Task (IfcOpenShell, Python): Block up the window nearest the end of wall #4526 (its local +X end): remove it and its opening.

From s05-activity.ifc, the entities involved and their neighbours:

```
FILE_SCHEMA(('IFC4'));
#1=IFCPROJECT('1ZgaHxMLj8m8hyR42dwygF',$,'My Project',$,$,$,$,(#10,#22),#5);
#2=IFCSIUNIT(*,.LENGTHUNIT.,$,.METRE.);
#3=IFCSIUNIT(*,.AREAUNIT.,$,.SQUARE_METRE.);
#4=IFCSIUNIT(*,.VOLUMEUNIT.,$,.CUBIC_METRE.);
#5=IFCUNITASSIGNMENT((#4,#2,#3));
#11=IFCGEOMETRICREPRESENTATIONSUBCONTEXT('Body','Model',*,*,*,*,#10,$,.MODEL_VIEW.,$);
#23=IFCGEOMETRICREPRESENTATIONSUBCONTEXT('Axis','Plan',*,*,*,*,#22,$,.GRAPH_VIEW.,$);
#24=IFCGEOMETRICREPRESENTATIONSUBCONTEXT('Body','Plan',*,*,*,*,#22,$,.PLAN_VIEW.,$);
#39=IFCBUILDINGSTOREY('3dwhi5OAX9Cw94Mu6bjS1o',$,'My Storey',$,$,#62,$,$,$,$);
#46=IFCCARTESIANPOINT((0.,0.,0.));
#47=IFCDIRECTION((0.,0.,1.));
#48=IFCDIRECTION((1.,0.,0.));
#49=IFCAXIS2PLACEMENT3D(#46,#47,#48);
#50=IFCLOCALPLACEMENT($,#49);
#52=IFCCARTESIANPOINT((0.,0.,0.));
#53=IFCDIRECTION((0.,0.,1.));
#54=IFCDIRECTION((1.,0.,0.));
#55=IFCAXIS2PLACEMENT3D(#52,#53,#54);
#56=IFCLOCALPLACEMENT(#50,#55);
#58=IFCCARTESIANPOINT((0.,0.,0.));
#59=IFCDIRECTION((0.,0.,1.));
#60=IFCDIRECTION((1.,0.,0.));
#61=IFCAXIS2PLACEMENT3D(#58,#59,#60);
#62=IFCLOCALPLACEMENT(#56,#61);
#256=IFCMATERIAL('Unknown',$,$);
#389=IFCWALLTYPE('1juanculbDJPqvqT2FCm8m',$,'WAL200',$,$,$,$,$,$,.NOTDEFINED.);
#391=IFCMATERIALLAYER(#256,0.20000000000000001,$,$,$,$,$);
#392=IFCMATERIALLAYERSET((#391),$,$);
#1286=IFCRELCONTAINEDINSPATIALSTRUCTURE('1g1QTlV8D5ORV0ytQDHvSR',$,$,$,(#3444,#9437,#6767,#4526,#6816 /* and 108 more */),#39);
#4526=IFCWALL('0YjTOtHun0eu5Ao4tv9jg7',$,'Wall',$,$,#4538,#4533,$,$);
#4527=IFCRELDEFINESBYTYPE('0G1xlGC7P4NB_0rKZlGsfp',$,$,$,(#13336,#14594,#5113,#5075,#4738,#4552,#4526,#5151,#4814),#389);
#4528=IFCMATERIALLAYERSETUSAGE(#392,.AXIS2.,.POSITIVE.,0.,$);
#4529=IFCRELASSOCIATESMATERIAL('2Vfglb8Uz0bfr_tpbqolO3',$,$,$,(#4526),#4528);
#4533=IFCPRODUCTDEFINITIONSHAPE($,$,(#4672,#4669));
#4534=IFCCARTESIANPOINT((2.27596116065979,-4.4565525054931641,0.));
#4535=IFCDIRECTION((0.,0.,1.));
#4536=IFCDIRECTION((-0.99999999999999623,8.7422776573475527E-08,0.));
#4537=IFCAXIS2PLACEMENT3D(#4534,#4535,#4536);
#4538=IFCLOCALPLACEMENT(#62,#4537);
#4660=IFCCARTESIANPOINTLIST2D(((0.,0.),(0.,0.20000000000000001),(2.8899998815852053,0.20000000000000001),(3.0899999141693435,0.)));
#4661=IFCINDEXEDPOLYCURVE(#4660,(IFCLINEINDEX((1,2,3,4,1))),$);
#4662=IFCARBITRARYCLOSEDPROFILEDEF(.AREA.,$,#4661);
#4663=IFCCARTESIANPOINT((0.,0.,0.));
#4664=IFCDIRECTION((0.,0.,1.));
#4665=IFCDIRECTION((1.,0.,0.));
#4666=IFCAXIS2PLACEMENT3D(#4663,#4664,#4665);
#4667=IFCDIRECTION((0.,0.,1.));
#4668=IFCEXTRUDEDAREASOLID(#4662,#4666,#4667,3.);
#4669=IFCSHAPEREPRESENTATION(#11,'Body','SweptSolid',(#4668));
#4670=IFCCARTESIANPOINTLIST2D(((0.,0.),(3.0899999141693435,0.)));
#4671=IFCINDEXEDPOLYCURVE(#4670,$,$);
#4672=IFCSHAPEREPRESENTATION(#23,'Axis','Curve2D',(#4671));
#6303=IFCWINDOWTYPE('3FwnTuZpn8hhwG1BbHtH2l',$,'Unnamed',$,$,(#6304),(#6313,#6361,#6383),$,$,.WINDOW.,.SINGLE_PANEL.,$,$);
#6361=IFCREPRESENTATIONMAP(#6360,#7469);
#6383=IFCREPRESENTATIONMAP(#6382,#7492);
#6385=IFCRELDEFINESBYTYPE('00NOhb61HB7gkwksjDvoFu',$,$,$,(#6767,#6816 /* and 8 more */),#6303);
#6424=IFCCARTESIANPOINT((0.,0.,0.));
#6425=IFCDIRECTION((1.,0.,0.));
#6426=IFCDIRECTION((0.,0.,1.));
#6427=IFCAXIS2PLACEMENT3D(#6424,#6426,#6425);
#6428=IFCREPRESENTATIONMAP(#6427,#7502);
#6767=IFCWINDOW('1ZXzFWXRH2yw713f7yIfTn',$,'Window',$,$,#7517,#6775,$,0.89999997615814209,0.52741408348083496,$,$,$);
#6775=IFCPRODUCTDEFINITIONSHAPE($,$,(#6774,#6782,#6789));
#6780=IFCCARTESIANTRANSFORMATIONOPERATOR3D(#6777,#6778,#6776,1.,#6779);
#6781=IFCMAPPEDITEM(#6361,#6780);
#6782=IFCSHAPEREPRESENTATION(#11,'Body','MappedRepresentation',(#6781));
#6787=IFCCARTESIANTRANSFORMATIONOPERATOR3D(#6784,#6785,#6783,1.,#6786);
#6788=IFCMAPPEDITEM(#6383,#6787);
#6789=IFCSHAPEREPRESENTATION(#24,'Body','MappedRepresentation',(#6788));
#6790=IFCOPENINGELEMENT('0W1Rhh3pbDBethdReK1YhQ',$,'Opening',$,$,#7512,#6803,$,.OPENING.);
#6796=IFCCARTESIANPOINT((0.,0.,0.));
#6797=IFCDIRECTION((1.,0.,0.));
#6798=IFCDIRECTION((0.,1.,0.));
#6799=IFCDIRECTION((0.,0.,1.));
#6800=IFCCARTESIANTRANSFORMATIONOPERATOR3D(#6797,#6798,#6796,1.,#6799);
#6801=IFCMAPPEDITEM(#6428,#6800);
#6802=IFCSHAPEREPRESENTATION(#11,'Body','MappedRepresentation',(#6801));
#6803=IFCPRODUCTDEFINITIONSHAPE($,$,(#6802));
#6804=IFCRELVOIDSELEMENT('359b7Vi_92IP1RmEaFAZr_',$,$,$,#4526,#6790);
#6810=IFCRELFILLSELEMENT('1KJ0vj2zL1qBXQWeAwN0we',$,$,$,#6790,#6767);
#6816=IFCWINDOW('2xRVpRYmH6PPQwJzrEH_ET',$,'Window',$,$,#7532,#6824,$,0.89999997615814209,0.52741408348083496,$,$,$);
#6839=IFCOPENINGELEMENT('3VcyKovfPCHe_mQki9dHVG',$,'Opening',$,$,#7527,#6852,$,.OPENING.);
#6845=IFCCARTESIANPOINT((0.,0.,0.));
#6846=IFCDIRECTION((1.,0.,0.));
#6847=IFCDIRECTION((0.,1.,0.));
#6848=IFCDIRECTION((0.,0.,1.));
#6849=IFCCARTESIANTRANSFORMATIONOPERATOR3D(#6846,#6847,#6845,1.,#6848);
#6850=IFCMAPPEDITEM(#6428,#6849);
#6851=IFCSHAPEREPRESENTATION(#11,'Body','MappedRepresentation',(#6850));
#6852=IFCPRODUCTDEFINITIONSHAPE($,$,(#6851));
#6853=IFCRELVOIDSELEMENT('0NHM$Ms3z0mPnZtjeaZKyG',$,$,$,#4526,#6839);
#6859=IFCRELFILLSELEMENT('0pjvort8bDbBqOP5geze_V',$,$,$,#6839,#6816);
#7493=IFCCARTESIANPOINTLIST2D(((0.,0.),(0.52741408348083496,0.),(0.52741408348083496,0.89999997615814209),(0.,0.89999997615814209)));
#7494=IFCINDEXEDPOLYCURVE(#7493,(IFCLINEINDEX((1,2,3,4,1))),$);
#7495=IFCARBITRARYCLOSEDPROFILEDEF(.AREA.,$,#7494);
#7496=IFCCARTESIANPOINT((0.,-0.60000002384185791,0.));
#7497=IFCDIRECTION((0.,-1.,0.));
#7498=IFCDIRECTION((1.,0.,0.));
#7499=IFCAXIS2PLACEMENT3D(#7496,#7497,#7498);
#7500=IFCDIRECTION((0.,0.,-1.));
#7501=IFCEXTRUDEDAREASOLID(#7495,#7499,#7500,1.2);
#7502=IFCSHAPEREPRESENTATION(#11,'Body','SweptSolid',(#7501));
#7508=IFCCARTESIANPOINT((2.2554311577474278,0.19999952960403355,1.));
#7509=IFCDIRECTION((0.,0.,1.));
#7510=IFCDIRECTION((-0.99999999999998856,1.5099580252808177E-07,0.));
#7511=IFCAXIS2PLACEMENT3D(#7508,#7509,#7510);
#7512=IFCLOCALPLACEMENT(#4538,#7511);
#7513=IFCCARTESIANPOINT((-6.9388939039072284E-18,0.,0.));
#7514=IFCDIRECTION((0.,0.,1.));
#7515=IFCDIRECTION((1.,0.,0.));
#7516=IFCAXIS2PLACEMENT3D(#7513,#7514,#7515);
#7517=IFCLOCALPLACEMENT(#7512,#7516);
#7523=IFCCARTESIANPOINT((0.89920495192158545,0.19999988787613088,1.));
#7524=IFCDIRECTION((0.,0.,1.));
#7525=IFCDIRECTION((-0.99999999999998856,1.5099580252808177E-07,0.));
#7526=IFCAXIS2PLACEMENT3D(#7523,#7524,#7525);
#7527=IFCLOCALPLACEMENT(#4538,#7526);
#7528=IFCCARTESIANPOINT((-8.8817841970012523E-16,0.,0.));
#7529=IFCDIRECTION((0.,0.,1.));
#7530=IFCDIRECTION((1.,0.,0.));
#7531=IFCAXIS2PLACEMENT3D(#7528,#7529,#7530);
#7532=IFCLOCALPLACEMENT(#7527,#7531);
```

```python
import ifcopenshell
import ifcopenshell.api.feature
import ifcopenshell.api.root
import ifcopenshell.geom
import ifcopenshell.util.shape

model = ifcopenshell.open("s05-activity.ifc")
settings = ifcopenshell.geom.settings()


def volume(element):
    """Net volume in cubic metres, openings subtracted."""
    shape = ifcopenshell.geom.create_shape(settings, element)
    return ifcopenshell.util.shape.get_volume(shape.geometry)


window = model.by_guid("1ZXzFWXRH2yw713f7yIfTn")
opening = window.FillsVoids[0].RelatingOpeningElement
wall = opening.VoidsElements[0].RelatingBuildingElement
before = volume(wall)

ifcopenshell.api.root.remove_product(model, product=window)
ifcopenshell.api.feature.remove_feature(model, feature=opening)

after = volume(wall)

print(f"wall volume {before:.3f} -> {after:.3f} m3")

model.write("s05-activity_updated.ifc")
```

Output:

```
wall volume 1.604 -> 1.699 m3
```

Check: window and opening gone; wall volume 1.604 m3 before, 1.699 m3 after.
